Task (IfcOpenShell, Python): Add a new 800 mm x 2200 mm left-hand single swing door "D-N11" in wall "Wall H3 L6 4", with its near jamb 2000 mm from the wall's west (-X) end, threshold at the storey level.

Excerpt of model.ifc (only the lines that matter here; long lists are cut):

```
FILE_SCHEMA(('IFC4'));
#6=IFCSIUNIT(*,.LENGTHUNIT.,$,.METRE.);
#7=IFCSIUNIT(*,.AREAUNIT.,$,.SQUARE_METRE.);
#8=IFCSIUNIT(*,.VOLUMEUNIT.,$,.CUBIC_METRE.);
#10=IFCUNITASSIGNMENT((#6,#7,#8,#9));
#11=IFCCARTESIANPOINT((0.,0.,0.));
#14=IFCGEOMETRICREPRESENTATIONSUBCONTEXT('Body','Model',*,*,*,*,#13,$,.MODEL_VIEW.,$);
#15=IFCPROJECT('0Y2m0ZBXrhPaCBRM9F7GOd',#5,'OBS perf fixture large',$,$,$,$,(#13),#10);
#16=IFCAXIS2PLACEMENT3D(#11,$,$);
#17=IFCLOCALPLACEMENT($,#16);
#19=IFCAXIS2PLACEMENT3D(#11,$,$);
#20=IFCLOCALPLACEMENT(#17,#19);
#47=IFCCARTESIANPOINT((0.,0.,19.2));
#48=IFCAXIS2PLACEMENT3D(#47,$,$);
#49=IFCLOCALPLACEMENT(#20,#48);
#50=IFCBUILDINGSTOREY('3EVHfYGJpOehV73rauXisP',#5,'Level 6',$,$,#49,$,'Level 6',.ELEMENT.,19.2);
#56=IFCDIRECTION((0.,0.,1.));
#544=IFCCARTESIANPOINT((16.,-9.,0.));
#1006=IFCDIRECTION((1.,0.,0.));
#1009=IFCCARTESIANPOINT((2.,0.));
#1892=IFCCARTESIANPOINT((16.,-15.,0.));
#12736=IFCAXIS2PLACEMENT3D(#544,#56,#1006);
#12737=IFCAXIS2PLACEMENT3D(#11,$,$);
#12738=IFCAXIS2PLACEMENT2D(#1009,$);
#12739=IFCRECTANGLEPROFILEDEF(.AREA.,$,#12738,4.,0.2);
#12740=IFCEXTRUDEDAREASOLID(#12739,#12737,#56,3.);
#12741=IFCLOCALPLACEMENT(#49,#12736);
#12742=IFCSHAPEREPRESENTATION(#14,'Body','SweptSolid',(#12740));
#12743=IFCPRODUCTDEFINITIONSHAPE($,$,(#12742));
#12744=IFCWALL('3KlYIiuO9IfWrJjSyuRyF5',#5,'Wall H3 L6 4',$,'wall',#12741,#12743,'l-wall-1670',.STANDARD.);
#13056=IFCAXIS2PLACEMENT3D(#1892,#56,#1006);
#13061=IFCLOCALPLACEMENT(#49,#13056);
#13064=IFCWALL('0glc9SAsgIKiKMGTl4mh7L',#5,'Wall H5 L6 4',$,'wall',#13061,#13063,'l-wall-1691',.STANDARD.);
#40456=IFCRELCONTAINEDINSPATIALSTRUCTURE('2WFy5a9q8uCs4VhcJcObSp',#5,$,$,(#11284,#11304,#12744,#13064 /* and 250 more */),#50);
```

```python
import numpy as np
import ifcopenshell
import ifcopenshell.api.feature
import ifcopenshell.api.geometry
import ifcopenshell.api.root
import ifcopenshell.api.spatial
import ifcopenshell.geom
import ifcopenshell.util.element
import ifcopenshell.util.placement
import ifcopenshell.util.representation
import ifcopenshell.util.shape
import ifcopenshell.util.unit

model = ifcopenshell.open("model.ifc")
unit_scale = ifcopenshell.util.unit.calculate_unit_scale(model)
settings = ifcopenshell.geom.settings()


def volume(element):
    """Net volume in cubic metres, openings subtracted."""
    shape = ifcopenshell.geom.create_shape(settings, element)
    return ifcopenshell.util.shape.get_volume(shape.geometry)


wall = model.by_guid("3KlYIiuO9IfWrJjSyuRyF5")
storey = ifcopenshell.util.element.get_container(wall, ifc_class="IfcBuildingStorey")
context = ifcopenshell.util.representation.get_context(model, "Model", "Body", "MODEL_VIEW")
before = volume(wall)

width, height, from_end, sill = 0.8, 2.2, 2, 0.0  # metres

# The wall runs along its own X axis, and the end named is its -X end.
wall_shape = ifcopenshell.geom.create_shape(settings, wall)
x, y, z = ifcopenshell.util.shape.get_vertices(wall_shape.geometry).T
start = x.min() + from_end
face, thickness = float(y.min()), float(y.max() - y.min())
wall_matrix = ifcopenshell.util.placement.get_local_placement(wall.ObjectPlacement)
level = ifcopenshell.util.placement.get_local_placement(storey.ObjectPlacement)[2, 3]


def in_wall(x, y):
    """Placement at x, y metres in the wall's axes, at sill height."""
    matrix = wall_matrix.copy()
    matrix[:, 3] = wall_matrix @ np.array([x / unit_scale, y / unit_scale, 0.0, 1.0])
    matrix[2, 3] = level + sill / unit_scale
    return matrix


# Opening: a box that overshoots both wall faces by 50 mm.
opening = ifcopenshell.api.root.create_entity(model, ifc_class="IfcOpeningElement", predefined_type="OPENING")
box = ifcopenshell.api.geometry.add_wall_representation(
    model, context=context, length=width, height=height, thickness=thickness + 0.1
)
ifcopenshell.api.geometry.assign_representation(model, product=opening, representation=box)
ifcopenshell.api.geometry.edit_object_placement(model, product=opening, matrix=in_wall(start, face - 0.05), is_si=False)
ifcopenshell.api.feature.add_feature(model, feature=opening, element=wall)

door = ifcopenshell.api.root.create_entity(model, ifc_class="IfcDoor", name="D-N11", predefined_type="DOOR")
door.OverallWidth, door.OverallHeight = width / unit_scale, height / unit_scale
door.OperationType = "SINGLE_SWING_LEFT"
body = ifcopenshell.api.geometry.add_door_representation(
    model,
    context=context,
    overall_width=door.OverallWidth,
    overall_height=door.OverallHeight,
    operation_type="SINGLE_SWING_LEFT",
    lining_properties={"LiningDepth": thickness / unit_scale, "ThresholdDepth": thickness / unit_scale},
)
ifcopenshell.api.geometry.assign_representation(model, product=door, representation=body)
ifcopenshell.api.spatial.assign_container(model, products=[door], relating_structure=storey)
ifcopenshell.api.feature.add_filling(model, opening=opening, element=door)

# The lining spans the wall, so the door starts at the wall face.
ifcopenshell.api.geometry.edit_object_placement(model, product=door, matrix=in_wall(start, face), is_si=False)

after = volume(wall)

print(f"wall volume {before:.3f} -> {after:.3f} m3")

model.write("model_updated.ifc")
```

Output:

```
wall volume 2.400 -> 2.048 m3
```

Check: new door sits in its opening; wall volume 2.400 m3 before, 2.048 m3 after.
